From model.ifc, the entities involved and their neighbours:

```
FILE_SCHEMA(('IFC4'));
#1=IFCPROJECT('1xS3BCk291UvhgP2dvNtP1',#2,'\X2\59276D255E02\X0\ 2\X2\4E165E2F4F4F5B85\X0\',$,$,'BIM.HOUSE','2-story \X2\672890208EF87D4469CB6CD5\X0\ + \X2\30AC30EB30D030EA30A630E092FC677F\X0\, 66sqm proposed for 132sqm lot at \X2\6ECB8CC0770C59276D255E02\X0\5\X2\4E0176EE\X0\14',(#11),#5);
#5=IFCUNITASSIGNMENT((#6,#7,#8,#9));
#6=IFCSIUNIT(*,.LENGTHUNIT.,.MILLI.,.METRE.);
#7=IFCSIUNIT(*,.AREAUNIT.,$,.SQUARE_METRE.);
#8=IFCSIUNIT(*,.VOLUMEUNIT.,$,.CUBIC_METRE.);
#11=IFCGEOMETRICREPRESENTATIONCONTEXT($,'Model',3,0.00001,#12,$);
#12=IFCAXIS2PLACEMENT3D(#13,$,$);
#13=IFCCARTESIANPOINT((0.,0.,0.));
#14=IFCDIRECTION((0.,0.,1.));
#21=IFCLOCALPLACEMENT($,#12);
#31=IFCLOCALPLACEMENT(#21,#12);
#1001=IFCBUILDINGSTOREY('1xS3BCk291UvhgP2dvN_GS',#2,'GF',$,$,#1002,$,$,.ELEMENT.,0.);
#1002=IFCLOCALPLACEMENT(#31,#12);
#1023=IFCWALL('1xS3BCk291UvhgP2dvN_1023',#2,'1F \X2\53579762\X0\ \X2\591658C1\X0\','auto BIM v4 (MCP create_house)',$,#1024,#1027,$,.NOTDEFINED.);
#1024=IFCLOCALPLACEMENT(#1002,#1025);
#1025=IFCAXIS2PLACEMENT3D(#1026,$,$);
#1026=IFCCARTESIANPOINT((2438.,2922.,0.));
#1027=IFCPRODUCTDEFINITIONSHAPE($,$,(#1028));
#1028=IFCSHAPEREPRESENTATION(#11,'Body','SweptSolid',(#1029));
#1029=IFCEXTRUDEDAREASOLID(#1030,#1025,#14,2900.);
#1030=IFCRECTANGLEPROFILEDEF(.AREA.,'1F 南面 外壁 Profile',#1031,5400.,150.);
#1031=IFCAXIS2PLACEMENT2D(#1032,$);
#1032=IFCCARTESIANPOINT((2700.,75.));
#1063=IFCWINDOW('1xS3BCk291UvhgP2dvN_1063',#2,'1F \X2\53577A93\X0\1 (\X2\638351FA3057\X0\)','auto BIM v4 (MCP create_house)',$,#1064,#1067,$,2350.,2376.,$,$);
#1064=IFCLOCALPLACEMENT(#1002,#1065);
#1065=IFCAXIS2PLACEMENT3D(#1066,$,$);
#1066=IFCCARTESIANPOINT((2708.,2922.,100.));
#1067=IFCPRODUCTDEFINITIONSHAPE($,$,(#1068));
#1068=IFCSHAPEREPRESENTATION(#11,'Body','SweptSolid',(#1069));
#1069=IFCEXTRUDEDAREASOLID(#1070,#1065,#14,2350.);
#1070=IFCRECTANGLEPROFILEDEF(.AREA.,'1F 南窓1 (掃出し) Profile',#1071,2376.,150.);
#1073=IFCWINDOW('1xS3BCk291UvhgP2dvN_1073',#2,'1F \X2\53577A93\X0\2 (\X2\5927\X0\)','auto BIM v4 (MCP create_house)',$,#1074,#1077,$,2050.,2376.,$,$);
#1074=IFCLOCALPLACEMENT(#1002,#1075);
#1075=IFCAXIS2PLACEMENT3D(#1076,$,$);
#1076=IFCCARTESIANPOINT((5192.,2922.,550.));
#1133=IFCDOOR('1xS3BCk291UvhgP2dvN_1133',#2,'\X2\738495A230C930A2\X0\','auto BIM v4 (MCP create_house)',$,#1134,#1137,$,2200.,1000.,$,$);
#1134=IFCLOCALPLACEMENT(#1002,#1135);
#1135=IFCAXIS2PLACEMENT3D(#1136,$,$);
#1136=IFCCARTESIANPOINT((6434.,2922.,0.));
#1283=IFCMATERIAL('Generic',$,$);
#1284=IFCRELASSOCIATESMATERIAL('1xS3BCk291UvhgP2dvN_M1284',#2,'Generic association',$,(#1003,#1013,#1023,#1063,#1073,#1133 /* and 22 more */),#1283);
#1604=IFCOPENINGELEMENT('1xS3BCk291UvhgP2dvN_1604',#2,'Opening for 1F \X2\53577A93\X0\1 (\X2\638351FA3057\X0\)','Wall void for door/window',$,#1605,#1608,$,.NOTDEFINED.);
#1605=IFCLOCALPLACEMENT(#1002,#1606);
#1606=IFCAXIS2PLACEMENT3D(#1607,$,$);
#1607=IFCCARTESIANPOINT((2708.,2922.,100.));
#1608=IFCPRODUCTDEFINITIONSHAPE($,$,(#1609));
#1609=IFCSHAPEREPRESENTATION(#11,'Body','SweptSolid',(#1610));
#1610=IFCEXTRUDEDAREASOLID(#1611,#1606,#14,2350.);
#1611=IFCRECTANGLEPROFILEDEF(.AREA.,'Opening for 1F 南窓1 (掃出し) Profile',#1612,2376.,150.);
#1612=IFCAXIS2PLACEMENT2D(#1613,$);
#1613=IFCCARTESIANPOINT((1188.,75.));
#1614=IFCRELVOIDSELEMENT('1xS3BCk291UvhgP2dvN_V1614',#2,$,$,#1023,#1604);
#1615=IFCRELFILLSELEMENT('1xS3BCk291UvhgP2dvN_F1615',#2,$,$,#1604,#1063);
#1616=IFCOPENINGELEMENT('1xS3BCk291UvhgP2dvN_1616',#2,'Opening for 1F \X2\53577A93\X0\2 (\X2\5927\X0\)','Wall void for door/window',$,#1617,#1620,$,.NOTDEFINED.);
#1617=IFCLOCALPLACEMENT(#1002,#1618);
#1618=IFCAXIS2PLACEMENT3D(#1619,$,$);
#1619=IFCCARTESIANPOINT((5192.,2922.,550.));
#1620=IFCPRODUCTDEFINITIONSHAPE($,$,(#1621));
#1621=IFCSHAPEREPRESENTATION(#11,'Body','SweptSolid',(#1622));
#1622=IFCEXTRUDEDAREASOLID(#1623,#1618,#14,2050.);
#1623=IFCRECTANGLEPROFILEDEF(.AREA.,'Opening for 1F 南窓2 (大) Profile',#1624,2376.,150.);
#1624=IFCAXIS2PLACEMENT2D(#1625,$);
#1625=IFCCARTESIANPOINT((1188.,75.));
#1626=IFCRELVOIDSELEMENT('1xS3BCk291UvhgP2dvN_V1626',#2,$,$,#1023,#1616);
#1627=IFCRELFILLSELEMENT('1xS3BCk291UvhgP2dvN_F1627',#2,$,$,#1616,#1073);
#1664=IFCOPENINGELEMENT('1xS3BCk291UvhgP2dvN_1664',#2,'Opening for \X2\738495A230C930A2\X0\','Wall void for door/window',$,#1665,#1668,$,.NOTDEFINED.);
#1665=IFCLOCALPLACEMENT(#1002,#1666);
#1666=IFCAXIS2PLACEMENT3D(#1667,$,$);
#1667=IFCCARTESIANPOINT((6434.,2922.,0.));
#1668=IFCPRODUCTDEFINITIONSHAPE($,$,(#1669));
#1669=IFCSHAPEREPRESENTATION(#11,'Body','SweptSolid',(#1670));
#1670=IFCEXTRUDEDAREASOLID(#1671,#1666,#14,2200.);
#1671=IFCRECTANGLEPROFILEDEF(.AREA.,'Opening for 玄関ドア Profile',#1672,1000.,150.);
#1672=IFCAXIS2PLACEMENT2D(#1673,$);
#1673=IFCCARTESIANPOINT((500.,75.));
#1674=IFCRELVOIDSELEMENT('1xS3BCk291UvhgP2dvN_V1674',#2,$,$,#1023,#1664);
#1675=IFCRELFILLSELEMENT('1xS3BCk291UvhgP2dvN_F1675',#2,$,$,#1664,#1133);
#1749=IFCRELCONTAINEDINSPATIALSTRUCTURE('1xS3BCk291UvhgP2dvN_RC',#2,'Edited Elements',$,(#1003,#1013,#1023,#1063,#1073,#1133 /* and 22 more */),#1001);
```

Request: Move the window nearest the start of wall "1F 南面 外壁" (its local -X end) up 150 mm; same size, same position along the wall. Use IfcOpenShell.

```python
import numpy as np
import ifcopenshell
import ifcopenshell.api.geometry
import ifcopenshell.util.placement
import ifcopenshell.util.unit

model = ifcopenshell.open("model.ifc")
unit_scale = ifcopenshell.util.unit.calculate_unit_scale(model)

window = model.by_guid("1xS3BCk291UvhgP2dvN_1063")
opening = window.FillsVoids[0].RelatingOpeningElement
dz = 0.15 / unit_scale

shift = np.array([0.0, 0.0, dz])
# The window is not placed relative to its opening, so move both.
for product in (opening, window):
    matrix = ifcopenshell.util.placement.get_local_placement(product.ObjectPlacement)
    matrix[:3, 3] += shift
    ifcopenshell.api.geometry.edit_object_placement(model, product=product, matrix=matrix, is_si=False)

print(f"moved by {dz * unit_scale:+.3f} m")

model.write("model_v2.ifc")
```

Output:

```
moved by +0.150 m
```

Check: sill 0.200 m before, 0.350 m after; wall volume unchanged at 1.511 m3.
